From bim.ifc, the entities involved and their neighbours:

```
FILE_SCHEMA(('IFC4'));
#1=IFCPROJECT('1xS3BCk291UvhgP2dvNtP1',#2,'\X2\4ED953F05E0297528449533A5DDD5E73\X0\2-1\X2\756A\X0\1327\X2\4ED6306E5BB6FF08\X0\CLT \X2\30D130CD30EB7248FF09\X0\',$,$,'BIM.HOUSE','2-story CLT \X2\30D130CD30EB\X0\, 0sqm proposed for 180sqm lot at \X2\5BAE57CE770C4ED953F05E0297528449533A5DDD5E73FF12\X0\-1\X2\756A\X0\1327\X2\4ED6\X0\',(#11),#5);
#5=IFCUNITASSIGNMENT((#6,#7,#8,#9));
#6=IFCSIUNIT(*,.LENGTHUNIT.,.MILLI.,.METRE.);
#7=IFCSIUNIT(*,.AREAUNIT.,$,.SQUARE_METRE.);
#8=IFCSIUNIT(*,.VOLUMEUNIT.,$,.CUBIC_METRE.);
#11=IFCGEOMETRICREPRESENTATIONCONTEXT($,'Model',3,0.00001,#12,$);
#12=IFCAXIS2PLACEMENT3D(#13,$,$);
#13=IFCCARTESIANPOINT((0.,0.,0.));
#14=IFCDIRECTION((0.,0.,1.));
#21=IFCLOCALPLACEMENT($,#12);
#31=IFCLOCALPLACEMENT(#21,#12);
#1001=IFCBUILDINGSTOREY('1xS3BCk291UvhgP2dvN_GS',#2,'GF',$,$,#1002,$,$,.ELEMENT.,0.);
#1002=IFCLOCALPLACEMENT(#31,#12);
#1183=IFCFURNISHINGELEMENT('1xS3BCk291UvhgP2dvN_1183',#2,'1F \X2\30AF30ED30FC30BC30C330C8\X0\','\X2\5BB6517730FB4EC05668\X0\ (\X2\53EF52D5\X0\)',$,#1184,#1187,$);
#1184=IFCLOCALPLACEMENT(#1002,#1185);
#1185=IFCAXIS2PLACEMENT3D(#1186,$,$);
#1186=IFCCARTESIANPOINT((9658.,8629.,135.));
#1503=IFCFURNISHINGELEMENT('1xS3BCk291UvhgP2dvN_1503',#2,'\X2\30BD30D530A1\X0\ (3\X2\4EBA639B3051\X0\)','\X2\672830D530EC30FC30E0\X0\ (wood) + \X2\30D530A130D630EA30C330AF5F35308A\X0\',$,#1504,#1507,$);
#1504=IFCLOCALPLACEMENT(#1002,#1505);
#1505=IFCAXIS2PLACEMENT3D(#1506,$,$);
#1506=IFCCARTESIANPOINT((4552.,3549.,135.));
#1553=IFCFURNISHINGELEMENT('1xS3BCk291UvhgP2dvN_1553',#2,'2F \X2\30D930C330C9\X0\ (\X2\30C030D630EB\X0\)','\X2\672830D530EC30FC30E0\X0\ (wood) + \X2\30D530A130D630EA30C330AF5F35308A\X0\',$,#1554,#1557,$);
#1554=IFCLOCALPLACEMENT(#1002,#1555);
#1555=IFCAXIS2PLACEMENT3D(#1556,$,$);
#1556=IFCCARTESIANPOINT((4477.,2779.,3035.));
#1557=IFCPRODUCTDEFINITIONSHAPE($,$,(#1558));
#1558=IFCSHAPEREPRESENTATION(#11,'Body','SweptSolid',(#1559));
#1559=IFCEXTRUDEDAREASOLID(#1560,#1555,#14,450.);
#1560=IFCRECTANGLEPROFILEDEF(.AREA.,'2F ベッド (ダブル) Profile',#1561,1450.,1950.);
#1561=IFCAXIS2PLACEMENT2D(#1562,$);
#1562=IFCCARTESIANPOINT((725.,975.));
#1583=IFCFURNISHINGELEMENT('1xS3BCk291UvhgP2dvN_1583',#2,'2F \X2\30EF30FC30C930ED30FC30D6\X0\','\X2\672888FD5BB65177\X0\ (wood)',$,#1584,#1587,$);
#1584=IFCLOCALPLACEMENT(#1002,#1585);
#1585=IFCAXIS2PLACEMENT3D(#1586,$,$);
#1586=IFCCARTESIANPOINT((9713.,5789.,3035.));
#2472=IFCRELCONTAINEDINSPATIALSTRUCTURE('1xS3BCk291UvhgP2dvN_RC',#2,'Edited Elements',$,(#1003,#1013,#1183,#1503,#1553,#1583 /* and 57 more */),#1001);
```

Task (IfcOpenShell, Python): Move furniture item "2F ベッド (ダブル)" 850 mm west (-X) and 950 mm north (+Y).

```python
import ifcopenshell
import ifcopenshell.api.geometry
import ifcopenshell.util.placement

model = ifcopenshell.open("bim.ifc")

item = model.by_guid("1xS3BCk291UvhgP2dvN_1553")
matrix = ifcopenshell.util.placement.get_local_placement(item.ObjectPlacement)
matrix[0, 3] -= 850.0
matrix[1, 3] += 950.0
ifcopenshell.api.geometry.edit_object_placement(model, product=item, matrix=matrix, is_si=False)

print(ifcopenshell.util.placement.get_local_placement(item.ObjectPlacement).round(3) + 0.0)

model.write("bim_updated.ifc")
```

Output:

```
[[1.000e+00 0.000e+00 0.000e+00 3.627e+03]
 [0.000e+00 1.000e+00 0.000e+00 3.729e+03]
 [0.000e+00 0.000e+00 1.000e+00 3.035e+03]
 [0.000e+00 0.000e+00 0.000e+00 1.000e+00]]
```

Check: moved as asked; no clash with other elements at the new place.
